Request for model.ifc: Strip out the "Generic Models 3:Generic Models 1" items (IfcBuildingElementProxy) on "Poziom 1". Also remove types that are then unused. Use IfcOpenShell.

First a look at what the model holds.

```python
import ifcopenshell
import ifcopenshell.util.element

model = ifcopenshell.open("model.ifc")
print(model.schema)
storey = next(s for s in model.by_type("IfcBuildingStorey") if s.Name == "Poziom 1")
proxies = [e for e in ifcopenshell.util.element.get_decomposition(storey) if e.is_a("IfcBuildingElementProxy")]
seen = {}
for e in proxies:
    element_type = ifcopenshell.util.element.get_type(e)
    name = element_type.Name if element_type not in (None, e) else None
    seen[name] = seen.get(name, 0) + 1
for name, count in sorted(seen.items(), key=str):
    print(count, "x", name)
```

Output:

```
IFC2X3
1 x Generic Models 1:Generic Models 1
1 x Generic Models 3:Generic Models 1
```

```python
import ifcopenshell
import ifcopenshell.api.root
import ifcopenshell.util.element

model = ifcopenshell.open("model.ifc")

storey = next(s for s in model.by_type("IfcBuildingStorey") if s.Name == "Poziom 1")
proxies = [e for e in ifcopenshell.util.element.get_decomposition(storey) if e.is_a("IfcBuildingElementProxy")]
targets = [e for e in proxies if (t := ifcopenshell.util.element.get_type(e)) not in (None, e) and t.Name == "Generic Models 3:Generic Models 1"]
types = {ifcopenshell.util.element.get_type(e) for e in targets} - {None, *targets}

for e in targets:
    ifcopenshell.api.root.remove_product(model, product=e)
print(len(targets), "removed")

unused = [t for t in types if not ifcopenshell.util.element.get_types(t)]
for t in unused:
    ifcopenshell.api.root.remove_product(model, product=t)
print(len(unused), "unused types removed")

model.write("model_rev.ifc")
```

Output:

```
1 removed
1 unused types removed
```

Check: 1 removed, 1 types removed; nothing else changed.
